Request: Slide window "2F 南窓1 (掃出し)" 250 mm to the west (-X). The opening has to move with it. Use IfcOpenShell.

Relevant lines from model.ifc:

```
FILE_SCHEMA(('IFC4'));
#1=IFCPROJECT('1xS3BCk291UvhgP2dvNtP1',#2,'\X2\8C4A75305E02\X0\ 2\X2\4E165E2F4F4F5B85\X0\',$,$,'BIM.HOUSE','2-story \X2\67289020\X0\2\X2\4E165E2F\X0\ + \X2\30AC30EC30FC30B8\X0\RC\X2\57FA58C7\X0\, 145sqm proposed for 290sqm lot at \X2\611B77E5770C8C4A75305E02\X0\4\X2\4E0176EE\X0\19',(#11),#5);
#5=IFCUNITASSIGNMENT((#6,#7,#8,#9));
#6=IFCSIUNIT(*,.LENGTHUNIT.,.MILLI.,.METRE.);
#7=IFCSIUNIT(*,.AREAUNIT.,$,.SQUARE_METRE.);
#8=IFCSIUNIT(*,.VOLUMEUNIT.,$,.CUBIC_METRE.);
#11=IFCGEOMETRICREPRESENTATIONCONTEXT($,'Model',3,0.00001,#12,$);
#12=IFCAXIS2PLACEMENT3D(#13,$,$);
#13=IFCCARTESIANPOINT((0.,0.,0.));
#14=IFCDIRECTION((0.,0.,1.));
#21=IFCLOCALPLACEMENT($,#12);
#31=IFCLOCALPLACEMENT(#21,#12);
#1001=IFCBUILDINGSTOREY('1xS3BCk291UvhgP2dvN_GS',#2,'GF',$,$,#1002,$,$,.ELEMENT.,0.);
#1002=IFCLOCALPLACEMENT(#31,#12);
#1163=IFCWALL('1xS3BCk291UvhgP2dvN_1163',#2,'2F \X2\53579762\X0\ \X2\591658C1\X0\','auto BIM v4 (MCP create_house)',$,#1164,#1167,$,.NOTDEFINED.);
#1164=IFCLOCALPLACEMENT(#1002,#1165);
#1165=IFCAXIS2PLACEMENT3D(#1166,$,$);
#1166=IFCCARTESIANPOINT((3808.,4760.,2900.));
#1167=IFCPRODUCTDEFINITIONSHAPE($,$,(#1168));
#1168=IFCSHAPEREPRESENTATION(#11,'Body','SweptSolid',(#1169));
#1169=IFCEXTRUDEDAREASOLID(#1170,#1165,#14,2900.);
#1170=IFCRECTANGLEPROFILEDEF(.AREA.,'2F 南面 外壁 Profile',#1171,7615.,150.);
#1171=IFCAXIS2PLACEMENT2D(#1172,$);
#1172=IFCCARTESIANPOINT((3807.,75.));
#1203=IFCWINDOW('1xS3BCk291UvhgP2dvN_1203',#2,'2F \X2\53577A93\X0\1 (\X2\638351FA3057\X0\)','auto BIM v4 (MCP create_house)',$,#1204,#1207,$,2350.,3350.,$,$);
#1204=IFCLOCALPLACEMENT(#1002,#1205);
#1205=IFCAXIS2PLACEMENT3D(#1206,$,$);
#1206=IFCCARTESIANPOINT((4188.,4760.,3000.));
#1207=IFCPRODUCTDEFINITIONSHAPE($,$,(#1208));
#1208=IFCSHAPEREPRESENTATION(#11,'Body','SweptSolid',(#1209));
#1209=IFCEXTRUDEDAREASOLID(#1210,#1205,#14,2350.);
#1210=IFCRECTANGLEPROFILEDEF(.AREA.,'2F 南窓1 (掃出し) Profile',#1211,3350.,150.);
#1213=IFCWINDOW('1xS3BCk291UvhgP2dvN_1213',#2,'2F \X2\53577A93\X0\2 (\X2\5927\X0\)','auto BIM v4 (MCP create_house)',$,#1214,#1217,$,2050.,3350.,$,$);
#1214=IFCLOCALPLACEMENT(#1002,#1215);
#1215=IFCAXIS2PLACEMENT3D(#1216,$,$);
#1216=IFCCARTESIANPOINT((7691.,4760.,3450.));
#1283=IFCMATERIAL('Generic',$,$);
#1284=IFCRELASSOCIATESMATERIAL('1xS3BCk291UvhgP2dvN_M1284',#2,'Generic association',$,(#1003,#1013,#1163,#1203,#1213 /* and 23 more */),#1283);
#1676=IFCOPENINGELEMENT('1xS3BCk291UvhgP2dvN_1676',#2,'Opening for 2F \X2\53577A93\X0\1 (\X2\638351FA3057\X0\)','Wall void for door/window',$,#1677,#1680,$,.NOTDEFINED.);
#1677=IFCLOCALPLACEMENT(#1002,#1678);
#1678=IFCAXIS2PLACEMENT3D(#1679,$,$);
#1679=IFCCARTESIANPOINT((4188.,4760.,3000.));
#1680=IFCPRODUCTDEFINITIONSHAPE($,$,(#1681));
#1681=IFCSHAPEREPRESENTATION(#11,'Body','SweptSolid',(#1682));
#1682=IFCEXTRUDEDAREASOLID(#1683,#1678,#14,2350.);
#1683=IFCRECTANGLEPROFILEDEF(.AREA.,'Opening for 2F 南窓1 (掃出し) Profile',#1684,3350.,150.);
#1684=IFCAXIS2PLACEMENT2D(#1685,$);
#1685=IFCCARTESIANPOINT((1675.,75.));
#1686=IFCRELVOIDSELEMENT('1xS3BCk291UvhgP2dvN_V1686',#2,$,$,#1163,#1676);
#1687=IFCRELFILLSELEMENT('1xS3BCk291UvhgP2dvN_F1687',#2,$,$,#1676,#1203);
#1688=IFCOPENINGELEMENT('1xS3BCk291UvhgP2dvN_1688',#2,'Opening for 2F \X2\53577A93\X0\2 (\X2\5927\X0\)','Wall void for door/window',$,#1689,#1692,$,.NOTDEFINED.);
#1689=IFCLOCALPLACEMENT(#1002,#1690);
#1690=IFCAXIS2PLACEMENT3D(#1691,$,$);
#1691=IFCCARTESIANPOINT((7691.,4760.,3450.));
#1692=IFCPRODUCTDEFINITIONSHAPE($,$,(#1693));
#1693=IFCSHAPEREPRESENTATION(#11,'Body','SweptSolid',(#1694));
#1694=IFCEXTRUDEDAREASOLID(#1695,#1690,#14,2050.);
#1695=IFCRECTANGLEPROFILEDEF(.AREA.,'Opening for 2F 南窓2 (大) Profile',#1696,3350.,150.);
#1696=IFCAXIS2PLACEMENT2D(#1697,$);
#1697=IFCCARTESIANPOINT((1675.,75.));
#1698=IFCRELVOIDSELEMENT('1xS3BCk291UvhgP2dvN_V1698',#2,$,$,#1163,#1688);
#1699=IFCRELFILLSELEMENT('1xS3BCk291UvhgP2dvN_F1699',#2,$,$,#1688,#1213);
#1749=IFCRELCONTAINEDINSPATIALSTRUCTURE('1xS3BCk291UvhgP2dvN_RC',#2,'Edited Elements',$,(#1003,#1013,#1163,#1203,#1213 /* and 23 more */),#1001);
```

```python
import ifcopenshell
import ifcopenshell.api.geometry
import ifcopenshell.util.placement
import ifcopenshell.util.unit

model = ifcopenshell.open("model.ifc")
unit_scale = ifcopenshell.util.unit.calculate_unit_scale(model)

window = model.by_guid("1xS3BCk291UvhgP2dvN_1203")
opening = window.FillsVoids[0].RelatingOpeningElement
wall = opening.VoidsElements[0].RelatingBuildingElement

wall_matrix = ifcopenshell.util.placement.get_local_placement(wall.ObjectPlacement)
shift = wall_matrix[:3, 0] * -0.25 / unit_scale
before = ifcopenshell.util.placement.get_local_placement(window.ObjectPlacement)[:3, 3].copy()

# The window is not placed relative to its opening, so move both.
for product in (opening, window):
    matrix = ifcopenshell.util.placement.get_local_placement(product.ObjectPlacement)
    matrix[:3, 3] += shift
    ifcopenshell.api.geometry.edit_object_placement(model, product=product, matrix=matrix, is_si=False)

after = ifcopenshell.util.placement.get_local_placement(window.ObjectPlacement)[:3, 3]
print("window moved by", (after - before).round(3) + 0.0)

model.write("model-out.ifc")
```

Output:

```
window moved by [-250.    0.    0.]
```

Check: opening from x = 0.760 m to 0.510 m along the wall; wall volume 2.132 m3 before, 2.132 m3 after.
